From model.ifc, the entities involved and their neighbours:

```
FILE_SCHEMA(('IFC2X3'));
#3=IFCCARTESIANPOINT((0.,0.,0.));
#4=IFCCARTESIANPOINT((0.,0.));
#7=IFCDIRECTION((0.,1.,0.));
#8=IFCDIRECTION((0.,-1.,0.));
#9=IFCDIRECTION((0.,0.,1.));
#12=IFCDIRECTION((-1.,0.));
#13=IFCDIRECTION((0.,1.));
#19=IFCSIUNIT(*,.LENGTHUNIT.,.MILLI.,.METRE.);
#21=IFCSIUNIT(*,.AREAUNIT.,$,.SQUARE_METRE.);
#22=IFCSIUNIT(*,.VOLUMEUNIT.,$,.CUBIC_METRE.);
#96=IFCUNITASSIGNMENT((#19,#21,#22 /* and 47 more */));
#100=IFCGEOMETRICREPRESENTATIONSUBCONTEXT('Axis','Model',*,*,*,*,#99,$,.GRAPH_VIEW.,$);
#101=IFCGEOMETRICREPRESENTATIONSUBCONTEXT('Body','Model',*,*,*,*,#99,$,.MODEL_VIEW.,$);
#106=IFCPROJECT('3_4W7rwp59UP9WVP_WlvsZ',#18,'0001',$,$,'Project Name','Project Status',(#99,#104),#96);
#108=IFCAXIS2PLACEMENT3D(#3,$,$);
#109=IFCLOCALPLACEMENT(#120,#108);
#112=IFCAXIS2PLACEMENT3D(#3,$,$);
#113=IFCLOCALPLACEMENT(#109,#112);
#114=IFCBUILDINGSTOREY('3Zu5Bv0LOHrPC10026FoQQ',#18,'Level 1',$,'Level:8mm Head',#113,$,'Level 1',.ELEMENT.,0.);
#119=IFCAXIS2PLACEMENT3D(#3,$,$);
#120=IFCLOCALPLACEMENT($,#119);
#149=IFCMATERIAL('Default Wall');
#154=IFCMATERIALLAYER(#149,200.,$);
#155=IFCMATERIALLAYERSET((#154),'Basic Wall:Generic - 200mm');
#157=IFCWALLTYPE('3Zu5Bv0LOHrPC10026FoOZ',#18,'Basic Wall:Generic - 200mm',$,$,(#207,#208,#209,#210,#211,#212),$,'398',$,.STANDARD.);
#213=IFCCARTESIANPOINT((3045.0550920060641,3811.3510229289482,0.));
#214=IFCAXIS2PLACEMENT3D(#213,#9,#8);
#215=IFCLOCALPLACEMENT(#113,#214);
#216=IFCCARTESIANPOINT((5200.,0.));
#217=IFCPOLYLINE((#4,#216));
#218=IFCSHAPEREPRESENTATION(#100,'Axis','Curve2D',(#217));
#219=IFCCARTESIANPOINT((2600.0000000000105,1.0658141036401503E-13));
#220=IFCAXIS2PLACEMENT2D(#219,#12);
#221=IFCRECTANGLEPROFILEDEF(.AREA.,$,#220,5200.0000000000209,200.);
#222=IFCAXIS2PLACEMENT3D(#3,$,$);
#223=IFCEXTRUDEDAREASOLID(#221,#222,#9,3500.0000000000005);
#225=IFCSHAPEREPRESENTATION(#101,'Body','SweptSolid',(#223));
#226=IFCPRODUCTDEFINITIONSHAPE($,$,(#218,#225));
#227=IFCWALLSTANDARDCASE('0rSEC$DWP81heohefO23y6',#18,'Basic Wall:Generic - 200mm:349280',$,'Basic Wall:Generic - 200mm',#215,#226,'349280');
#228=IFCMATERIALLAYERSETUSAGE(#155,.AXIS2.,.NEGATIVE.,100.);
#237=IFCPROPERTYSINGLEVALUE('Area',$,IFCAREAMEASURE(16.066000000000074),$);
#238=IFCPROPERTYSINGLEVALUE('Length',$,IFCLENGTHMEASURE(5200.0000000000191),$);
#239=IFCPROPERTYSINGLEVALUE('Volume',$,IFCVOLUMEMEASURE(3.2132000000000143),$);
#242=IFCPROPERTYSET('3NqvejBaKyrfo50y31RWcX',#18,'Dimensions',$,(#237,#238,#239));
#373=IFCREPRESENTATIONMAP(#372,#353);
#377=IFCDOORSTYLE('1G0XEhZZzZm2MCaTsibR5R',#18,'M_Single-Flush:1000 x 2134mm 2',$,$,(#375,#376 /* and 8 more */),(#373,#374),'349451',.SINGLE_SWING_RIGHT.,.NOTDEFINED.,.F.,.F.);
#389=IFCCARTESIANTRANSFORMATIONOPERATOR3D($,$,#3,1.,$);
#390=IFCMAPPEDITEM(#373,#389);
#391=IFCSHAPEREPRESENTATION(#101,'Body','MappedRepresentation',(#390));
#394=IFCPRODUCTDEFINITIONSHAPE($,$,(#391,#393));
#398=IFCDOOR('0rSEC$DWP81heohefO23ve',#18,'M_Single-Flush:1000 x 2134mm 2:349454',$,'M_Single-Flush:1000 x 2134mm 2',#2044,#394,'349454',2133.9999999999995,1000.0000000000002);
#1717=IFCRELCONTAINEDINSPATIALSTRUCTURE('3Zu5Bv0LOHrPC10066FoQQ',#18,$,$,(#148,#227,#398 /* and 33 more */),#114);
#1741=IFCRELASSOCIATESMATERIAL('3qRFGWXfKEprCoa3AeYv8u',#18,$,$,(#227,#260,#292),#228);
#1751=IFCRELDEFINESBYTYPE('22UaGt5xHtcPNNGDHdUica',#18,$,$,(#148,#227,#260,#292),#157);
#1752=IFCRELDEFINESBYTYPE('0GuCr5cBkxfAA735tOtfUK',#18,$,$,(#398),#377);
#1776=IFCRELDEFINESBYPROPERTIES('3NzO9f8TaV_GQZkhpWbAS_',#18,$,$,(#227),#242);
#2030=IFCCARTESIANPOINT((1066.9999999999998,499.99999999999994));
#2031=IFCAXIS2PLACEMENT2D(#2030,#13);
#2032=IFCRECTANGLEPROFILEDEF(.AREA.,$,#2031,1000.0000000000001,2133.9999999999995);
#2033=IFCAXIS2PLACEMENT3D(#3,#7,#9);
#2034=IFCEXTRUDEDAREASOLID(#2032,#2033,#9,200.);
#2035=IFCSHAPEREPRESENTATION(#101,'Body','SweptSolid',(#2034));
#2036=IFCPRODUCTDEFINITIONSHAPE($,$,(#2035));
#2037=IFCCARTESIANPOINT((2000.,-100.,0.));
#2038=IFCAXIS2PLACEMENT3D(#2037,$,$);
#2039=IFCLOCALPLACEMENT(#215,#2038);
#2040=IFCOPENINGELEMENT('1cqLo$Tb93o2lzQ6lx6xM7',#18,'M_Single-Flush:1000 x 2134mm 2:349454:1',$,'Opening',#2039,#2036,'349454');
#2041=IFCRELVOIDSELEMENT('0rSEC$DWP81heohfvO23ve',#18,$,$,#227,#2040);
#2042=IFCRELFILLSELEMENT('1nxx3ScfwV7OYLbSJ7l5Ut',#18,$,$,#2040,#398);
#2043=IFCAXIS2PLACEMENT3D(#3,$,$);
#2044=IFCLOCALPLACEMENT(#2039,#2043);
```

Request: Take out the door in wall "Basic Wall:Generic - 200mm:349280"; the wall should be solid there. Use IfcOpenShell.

```python
import ifcopenshell
import ifcopenshell.api.feature
import ifcopenshell.api.pset
import ifcopenshell.api.root
import ifcopenshell.geom
import ifcopenshell.util.element
import ifcopenshell.util.shape
import ifcopenshell.util.unit

model = ifcopenshell.open("model.ifc")
area_scale = ifcopenshell.util.unit.calculate_unit_scale(model, "AREAUNIT")
volume_scale = ifcopenshell.util.unit.calculate_unit_scale(model, "VOLUMEUNIT")
settings = ifcopenshell.geom.settings()


def volume(element):
    """Net volume in cubic metres, openings subtracted."""
    shape = ifcopenshell.geom.create_shape(settings, element)
    return ifcopenshell.util.shape.get_volume(shape.geometry)


door = model.by_guid("0rSEC$DWP81heohefO23ve")
opening = door.FillsVoids[0].RelatingOpeningElement
wall = opening.VoidsElements[0].RelatingBuildingElement
before = volume(wall)

ifcopenshell.api.root.remove_product(model, product=door)
ifcopenshell.api.feature.remove_feature(model, feature=opening)

after = volume(wall)
thickness = 0.2  # wall thickness in metres

# Update the wall's stored quantities.
pset = model.by_id(ifcopenshell.util.element.get_pset(wall, "Dimensions", should_inherit=False)["id"])
ifcopenshell.api.pset.edit_pset(model, pset=pset, properties={
    "Area": model.create_entity("IfcAreaMeasure", after / thickness / area_scale),
    "Volume": model.create_entity("IfcVolumeMeasure", after / volume_scale),
})

print(f"wall volume {before:.3f} -> {after:.3f} m3")

model.write("model_edited.ifc")
```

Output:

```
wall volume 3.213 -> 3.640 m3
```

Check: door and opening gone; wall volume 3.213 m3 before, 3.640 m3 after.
